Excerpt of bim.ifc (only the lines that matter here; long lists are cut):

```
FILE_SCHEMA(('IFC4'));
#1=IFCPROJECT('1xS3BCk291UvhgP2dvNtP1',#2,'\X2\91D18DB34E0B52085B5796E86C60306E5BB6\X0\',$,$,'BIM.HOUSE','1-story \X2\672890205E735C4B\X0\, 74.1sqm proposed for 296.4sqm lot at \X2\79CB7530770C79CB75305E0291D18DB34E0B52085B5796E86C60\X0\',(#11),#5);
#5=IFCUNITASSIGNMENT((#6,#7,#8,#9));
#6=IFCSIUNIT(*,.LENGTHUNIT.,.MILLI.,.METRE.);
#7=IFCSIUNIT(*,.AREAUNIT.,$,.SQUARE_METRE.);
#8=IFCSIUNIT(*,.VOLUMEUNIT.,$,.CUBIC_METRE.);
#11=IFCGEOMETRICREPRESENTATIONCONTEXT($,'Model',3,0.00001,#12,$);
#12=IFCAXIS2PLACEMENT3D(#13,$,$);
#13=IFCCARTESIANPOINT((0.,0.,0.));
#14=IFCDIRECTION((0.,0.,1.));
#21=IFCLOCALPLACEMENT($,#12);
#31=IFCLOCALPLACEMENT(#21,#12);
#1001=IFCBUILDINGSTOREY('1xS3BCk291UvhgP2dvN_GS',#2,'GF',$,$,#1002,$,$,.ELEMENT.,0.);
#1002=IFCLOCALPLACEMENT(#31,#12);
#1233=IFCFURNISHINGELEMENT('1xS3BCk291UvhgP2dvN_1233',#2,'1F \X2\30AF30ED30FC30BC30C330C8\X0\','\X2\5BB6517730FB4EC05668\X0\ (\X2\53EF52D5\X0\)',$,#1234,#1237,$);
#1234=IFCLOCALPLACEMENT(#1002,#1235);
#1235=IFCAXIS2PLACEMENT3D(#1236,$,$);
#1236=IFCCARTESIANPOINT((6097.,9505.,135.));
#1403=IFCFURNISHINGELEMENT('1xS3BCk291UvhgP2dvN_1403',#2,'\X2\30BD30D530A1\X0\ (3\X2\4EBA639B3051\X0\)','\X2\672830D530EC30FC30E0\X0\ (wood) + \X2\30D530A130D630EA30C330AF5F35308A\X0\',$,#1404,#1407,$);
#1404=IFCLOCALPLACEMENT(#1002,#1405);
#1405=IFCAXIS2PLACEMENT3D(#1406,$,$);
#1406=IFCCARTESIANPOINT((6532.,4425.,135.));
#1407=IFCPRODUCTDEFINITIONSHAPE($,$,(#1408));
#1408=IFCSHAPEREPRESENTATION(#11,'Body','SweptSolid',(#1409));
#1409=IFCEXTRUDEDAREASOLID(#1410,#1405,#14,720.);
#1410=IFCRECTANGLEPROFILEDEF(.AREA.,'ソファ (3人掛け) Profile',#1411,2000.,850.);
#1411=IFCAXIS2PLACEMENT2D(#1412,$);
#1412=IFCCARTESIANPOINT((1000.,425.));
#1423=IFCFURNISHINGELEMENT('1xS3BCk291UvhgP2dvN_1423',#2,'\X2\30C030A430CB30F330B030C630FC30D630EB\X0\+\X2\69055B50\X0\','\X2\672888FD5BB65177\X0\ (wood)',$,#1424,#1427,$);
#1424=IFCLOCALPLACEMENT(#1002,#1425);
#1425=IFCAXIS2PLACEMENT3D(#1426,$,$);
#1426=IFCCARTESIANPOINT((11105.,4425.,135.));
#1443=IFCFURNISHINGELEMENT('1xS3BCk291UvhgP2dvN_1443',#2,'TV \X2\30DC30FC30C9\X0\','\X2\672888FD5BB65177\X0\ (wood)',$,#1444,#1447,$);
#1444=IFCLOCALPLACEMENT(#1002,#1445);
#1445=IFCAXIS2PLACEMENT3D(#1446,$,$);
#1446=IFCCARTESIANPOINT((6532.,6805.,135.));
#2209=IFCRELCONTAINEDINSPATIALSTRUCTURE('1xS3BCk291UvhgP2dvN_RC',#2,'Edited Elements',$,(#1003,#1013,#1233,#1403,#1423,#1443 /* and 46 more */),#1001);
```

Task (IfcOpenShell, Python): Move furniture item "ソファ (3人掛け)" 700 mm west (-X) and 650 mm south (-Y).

```python
import ifcopenshell
import ifcopenshell.api.geometry
import ifcopenshell.util.placement
import ifcopenshell.util.unit

model = ifcopenshell.open("bim.ifc")
unit_scale = ifcopenshell.util.unit.calculate_unit_scale(model)

item = model.by_guid("1xS3BCk291UvhgP2dvN_1403")
matrix = ifcopenshell.util.placement.get_local_placement(item.ObjectPlacement)
matrix[0, 3] -= 0.7 / unit_scale
matrix[1, 3] -= 0.65 / unit_scale
ifcopenshell.api.geometry.edit_object_placement(model, product=item, matrix=matrix, is_si=False)

print(ifcopenshell.util.placement.get_local_placement(item.ObjectPlacement).round(3) + 0.0)

model.write("bim_rev.ifc")
```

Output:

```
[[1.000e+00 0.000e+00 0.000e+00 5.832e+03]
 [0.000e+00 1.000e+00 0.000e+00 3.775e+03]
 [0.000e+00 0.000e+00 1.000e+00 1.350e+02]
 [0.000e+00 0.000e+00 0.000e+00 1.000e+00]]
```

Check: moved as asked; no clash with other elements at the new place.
